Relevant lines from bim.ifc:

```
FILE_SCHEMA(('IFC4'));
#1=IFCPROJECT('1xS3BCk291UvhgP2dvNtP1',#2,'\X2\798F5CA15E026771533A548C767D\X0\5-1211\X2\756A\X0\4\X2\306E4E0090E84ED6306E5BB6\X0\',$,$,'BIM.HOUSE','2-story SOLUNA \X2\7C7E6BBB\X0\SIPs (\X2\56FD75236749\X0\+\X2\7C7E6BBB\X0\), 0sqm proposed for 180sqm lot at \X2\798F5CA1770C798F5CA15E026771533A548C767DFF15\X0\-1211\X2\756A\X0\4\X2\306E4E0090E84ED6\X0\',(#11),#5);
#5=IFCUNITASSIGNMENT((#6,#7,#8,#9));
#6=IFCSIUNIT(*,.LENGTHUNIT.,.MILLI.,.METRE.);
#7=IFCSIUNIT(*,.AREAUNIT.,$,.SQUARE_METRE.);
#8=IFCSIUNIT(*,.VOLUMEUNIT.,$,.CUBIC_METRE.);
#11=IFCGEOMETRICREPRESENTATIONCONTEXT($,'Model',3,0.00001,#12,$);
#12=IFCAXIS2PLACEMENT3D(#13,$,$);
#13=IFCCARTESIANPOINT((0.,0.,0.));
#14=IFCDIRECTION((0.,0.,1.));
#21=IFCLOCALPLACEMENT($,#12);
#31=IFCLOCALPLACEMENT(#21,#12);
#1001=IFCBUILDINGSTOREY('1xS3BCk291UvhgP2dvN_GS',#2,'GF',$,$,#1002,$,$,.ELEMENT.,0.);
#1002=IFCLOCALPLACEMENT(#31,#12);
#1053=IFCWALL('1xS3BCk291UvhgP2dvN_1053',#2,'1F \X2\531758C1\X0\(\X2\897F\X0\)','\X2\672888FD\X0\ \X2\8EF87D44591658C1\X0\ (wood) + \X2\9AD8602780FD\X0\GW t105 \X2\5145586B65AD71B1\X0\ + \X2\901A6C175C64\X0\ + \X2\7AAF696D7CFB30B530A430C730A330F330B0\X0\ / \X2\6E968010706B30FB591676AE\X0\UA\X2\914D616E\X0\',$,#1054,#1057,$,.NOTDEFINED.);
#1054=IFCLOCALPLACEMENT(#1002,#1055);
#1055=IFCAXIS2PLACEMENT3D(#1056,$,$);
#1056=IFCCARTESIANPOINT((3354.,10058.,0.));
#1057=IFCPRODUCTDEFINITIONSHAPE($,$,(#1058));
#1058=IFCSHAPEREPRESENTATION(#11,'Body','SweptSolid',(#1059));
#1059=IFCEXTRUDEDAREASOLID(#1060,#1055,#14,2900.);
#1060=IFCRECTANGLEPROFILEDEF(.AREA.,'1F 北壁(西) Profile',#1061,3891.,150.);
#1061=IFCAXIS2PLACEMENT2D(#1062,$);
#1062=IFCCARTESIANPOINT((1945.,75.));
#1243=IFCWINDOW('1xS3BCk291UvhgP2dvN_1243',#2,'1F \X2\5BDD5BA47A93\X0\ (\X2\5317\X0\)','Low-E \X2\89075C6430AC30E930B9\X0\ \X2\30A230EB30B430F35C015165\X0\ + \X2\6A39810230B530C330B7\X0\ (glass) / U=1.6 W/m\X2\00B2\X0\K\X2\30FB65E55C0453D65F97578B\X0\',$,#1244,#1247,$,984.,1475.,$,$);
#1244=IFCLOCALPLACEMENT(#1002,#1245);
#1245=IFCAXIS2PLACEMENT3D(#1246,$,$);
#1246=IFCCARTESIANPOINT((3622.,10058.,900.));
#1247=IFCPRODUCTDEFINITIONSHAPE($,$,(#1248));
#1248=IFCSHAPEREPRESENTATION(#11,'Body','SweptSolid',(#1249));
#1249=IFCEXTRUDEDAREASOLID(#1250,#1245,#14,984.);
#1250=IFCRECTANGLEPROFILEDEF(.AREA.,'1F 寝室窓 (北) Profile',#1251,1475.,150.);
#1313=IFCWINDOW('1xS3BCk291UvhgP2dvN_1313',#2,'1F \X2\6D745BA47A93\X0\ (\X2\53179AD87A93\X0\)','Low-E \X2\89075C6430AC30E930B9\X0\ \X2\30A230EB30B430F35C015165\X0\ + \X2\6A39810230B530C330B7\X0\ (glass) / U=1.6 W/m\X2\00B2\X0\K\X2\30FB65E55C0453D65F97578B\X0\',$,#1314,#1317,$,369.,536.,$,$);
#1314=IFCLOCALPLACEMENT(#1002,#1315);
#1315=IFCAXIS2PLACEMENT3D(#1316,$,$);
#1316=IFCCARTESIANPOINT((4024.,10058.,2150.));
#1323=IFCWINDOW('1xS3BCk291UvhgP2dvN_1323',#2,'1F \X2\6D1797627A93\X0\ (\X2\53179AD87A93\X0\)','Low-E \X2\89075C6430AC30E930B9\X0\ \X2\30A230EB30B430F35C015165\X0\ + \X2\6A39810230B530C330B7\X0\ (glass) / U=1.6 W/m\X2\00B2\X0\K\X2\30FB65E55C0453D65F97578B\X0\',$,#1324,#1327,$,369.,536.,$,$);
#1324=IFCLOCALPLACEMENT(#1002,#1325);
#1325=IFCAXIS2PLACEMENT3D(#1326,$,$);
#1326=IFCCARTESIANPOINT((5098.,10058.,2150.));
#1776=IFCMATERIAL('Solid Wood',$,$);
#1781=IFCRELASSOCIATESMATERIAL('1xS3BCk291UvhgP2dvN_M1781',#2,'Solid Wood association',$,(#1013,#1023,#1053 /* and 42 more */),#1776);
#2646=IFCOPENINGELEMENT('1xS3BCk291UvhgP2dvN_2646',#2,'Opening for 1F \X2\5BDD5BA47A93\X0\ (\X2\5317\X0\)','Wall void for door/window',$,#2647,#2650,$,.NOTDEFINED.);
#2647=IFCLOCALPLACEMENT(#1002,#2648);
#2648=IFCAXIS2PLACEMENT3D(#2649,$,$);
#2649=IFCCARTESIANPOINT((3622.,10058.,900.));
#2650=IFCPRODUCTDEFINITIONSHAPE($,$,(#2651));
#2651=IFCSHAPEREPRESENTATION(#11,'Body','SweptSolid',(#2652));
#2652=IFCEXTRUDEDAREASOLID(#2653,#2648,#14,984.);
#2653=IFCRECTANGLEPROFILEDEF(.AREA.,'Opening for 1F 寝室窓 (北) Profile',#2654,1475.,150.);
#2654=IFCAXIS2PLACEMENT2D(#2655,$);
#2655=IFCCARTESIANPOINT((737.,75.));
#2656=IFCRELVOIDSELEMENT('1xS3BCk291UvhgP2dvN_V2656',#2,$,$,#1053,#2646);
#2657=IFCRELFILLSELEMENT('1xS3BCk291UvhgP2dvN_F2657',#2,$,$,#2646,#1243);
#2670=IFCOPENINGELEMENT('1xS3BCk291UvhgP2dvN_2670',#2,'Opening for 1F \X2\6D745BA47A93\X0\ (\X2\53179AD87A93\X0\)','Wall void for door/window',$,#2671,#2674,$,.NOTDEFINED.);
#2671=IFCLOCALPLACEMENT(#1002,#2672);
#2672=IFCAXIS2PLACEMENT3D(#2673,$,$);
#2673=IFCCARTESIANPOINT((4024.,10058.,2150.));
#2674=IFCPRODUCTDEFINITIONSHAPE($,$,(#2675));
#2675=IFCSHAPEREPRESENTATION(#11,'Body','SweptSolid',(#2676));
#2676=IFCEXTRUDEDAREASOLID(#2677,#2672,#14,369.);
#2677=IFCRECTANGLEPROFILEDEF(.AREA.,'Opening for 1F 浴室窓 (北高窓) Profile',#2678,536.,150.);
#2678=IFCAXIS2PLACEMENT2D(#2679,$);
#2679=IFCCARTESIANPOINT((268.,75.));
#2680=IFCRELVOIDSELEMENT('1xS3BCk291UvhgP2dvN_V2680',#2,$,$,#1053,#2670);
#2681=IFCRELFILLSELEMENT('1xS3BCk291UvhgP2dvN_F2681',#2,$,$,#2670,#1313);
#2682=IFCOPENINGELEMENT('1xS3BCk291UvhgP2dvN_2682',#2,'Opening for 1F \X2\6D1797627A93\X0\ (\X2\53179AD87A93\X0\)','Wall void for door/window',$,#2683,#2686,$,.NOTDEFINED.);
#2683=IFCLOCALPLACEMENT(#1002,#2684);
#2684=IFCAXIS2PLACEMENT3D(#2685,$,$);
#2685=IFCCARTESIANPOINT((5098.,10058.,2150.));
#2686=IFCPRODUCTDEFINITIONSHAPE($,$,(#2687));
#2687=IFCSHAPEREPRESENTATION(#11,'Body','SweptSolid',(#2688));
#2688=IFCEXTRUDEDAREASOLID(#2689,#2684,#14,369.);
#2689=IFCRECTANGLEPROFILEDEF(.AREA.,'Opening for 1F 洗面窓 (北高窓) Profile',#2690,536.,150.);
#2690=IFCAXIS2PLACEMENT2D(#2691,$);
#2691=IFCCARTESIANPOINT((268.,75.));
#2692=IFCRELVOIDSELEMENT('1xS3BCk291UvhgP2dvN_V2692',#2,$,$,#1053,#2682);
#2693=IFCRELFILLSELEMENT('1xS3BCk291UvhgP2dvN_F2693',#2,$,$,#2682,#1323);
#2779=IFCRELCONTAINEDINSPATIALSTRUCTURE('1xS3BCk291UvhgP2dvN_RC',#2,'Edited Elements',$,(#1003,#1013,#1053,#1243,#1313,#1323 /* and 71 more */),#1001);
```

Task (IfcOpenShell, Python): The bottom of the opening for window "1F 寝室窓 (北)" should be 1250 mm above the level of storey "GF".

```python
import numpy as np
import ifcopenshell
import ifcopenshell.api.geometry
import ifcopenshell.geom
import ifcopenshell.util.element
import ifcopenshell.util.placement
import ifcopenshell.util.shape
import ifcopenshell.util.unit

model = ifcopenshell.open("bim.ifc")
unit_scale = ifcopenshell.util.unit.calculate_unit_scale(model)

window = model.by_guid("1xS3BCk291UvhgP2dvN_1243")
opening = window.FillsVoids[0].RelatingOpeningElement
storey = ifcopenshell.util.element.get_container(window, ifc_class="IfcBuildingStorey")
level = ifcopenshell.util.placement.get_local_placement(storey.ObjectPlacement)[2, 3]

# The opening's origin need not be at the sill, so measure its lowest point.
shape = ifcopenshell.geom.create_shape(ifcopenshell.geom.settings(), opening)
bottom = ifcopenshell.util.shape.get_shape_bottom_elevation(shape, shape.geometry) / unit_scale
dz = level + 1.25 / unit_scale - bottom

shift = np.array([0.0, 0.0, dz])
# The window is not placed relative to its opening, so move both.
for product in (opening, window):
    matrix = ifcopenshell.util.placement.get_local_placement(product.ObjectPlacement)
    matrix[:3, 3] += shift
    ifcopenshell.api.geometry.edit_object_placement(model, product=product, matrix=matrix, is_si=False)

print(f"moved by {dz * unit_scale:+.3f} m")

model.write("bim_rev.ifc")
```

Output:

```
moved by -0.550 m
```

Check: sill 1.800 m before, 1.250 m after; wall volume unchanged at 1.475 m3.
